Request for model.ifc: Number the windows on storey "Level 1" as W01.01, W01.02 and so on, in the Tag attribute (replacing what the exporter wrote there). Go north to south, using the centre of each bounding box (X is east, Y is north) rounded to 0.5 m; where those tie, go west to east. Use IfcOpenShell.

First a look at what the model holds.

```python
import ifcopenshell
import ifcopenshell.util.element
import ifcopenshell.util.placement

model = ifcopenshell.open("model.ifc")
print(model.schema)
storey = next(s for s in model.by_type("IfcBuildingStorey") if s.Name == "Level 1")
windows = [e for e in ifcopenshell.util.element.get_decomposition(storey) if e.is_a("IfcWindow")]
for e in sorted(windows, key=lambda e: e.id()):
    origin = ifcopenshell.util.placement.get_local_placement(e.ObjectPlacement)[:3, 3]
    print(e.id(), e.Tag, e.Name, origin.round(2) + 0.0, sep=" | ")
```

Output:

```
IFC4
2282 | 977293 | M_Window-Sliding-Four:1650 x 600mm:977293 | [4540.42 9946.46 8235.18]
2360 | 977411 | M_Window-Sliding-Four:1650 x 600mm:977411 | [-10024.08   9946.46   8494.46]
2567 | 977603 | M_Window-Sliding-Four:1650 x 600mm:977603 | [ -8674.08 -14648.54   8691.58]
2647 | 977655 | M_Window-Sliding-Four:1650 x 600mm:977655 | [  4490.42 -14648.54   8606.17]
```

```python
import ifcopenshell
import ifcopenshell.geom
import ifcopenshell.util.element
import ifcopenshell.util.shape

model = ifcopenshell.open("model.ifc")
settings = ifcopenshell.geom.settings()
settings.set("use-world-coords", True)


def centre(element):
    shape = ifcopenshell.geom.create_shape(settings, element)
    return ifcopenshell.util.shape.get_bbox_centroid(shape.geometry)


storey = next(s for s in model.by_type("IfcBuildingStorey") if s.Name == "Level 1")
windows = [e for e in ifcopenshell.util.element.get_decomposition(storey) if e.is_a("IfcWindow")]

# Insertion points can sit at a corner or the storey origin, so sort by the geometry (in metres).
centres = {e: centre(e) for e in windows}
windows.sort(key=lambda e: (-round(centres[e][1] / 0.5), centres[e][0]))

for i, e in enumerate(windows, start=1):
    number = f"W01.{i:02d}"
    e.Tag = number
    print(e.id(), number)

model.write("model_updated.ifc")
```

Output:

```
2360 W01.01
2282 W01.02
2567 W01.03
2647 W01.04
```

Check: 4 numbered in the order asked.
